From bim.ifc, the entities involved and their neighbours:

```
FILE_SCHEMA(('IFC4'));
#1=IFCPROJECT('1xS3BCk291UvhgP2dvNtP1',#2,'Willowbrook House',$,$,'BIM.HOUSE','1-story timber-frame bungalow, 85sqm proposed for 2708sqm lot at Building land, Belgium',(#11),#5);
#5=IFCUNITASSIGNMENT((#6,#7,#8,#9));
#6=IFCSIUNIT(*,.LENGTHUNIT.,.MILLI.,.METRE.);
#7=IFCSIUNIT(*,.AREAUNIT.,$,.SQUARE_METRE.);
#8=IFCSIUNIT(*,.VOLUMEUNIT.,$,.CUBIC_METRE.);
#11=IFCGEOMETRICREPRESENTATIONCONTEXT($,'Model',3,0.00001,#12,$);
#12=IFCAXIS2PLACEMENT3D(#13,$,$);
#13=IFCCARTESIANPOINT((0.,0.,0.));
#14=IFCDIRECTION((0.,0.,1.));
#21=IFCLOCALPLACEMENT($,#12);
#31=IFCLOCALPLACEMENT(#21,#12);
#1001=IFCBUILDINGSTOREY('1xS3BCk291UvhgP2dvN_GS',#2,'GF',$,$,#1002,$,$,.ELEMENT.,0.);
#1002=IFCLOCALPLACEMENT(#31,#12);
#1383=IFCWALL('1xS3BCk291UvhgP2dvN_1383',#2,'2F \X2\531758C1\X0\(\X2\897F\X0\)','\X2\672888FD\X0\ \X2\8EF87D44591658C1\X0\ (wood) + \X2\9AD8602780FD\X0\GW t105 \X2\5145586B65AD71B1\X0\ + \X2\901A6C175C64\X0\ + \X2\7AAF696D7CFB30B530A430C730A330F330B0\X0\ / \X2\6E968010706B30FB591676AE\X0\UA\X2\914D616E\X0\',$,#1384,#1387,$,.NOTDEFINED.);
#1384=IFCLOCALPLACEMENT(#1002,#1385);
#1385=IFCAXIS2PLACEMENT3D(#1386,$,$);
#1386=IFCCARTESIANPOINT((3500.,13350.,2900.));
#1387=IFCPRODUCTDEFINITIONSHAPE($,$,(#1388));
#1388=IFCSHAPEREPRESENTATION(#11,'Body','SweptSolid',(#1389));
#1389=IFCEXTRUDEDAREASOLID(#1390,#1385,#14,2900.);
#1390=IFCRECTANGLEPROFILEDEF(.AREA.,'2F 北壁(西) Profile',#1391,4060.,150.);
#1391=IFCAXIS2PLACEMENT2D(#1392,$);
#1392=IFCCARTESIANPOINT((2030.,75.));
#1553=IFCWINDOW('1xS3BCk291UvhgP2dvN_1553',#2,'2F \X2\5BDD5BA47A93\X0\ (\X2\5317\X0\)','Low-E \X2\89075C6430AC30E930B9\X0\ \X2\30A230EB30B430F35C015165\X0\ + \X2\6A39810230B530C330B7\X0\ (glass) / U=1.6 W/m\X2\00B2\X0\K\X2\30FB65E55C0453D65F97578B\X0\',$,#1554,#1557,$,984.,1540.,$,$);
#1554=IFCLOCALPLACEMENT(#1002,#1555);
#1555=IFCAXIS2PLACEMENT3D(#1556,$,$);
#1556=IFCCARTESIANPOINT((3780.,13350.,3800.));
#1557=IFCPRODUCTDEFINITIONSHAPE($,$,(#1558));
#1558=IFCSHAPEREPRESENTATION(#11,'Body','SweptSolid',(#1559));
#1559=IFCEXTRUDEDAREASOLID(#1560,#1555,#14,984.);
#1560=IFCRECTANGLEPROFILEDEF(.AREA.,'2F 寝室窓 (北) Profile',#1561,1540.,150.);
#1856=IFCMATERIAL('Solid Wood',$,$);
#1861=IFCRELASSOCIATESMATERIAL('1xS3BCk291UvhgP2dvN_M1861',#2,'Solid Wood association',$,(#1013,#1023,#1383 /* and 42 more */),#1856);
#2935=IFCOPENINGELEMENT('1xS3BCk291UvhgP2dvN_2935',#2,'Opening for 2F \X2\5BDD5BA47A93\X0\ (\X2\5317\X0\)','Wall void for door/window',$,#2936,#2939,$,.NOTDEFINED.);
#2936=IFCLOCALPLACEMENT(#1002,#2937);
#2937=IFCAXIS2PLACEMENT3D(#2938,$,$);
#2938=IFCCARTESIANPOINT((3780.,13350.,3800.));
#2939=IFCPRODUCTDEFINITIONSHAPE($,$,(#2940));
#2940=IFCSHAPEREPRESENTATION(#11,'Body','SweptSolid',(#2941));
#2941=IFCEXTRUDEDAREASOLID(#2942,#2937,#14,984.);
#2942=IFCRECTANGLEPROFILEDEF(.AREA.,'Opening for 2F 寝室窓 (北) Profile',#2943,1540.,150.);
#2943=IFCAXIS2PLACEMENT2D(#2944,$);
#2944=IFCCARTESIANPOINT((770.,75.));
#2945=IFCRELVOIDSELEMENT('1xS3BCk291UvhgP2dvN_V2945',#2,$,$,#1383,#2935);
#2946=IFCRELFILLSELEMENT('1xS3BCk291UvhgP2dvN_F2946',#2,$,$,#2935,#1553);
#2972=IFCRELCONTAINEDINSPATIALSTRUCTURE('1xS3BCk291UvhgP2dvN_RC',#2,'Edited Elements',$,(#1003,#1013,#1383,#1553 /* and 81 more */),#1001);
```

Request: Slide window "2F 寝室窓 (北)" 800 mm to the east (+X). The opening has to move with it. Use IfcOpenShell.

```python
import ifcopenshell
import ifcopenshell.api.geometry
import ifcopenshell.util.placement
import ifcopenshell.util.unit

model = ifcopenshell.open("bim.ifc")
unit_scale = ifcopenshell.util.unit.calculate_unit_scale(model)

window = model.by_guid("1xS3BCk291UvhgP2dvN_1553")
opening = window.FillsVoids[0].RelatingOpeningElement
wall = opening.VoidsElements[0].RelatingBuildingElement

wall_matrix = ifcopenshell.util.placement.get_local_placement(wall.ObjectPlacement)
shift = wall_matrix[:3, 0] * 0.8 / unit_scale
before = ifcopenshell.util.placement.get_local_placement(window.ObjectPlacement)[:3, 3].copy()

# The window is not placed relative to its opening, so move both.
for product in (opening, window):
    matrix = ifcopenshell.util.placement.get_local_placement(product.ObjectPlacement)
    matrix[:3, 3] += shift
    ifcopenshell.api.geometry.edit_object_placement(model, product=product, matrix=matrix, is_si=False)

after = ifcopenshell.util.placement.get_local_placement(window.ObjectPlacement)[:3, 3]
print("window moved by", (after - before).round(3) + 0.0)

model.write("bim_updated.ifc")
```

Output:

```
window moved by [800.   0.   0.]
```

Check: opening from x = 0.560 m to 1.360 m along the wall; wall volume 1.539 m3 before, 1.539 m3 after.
